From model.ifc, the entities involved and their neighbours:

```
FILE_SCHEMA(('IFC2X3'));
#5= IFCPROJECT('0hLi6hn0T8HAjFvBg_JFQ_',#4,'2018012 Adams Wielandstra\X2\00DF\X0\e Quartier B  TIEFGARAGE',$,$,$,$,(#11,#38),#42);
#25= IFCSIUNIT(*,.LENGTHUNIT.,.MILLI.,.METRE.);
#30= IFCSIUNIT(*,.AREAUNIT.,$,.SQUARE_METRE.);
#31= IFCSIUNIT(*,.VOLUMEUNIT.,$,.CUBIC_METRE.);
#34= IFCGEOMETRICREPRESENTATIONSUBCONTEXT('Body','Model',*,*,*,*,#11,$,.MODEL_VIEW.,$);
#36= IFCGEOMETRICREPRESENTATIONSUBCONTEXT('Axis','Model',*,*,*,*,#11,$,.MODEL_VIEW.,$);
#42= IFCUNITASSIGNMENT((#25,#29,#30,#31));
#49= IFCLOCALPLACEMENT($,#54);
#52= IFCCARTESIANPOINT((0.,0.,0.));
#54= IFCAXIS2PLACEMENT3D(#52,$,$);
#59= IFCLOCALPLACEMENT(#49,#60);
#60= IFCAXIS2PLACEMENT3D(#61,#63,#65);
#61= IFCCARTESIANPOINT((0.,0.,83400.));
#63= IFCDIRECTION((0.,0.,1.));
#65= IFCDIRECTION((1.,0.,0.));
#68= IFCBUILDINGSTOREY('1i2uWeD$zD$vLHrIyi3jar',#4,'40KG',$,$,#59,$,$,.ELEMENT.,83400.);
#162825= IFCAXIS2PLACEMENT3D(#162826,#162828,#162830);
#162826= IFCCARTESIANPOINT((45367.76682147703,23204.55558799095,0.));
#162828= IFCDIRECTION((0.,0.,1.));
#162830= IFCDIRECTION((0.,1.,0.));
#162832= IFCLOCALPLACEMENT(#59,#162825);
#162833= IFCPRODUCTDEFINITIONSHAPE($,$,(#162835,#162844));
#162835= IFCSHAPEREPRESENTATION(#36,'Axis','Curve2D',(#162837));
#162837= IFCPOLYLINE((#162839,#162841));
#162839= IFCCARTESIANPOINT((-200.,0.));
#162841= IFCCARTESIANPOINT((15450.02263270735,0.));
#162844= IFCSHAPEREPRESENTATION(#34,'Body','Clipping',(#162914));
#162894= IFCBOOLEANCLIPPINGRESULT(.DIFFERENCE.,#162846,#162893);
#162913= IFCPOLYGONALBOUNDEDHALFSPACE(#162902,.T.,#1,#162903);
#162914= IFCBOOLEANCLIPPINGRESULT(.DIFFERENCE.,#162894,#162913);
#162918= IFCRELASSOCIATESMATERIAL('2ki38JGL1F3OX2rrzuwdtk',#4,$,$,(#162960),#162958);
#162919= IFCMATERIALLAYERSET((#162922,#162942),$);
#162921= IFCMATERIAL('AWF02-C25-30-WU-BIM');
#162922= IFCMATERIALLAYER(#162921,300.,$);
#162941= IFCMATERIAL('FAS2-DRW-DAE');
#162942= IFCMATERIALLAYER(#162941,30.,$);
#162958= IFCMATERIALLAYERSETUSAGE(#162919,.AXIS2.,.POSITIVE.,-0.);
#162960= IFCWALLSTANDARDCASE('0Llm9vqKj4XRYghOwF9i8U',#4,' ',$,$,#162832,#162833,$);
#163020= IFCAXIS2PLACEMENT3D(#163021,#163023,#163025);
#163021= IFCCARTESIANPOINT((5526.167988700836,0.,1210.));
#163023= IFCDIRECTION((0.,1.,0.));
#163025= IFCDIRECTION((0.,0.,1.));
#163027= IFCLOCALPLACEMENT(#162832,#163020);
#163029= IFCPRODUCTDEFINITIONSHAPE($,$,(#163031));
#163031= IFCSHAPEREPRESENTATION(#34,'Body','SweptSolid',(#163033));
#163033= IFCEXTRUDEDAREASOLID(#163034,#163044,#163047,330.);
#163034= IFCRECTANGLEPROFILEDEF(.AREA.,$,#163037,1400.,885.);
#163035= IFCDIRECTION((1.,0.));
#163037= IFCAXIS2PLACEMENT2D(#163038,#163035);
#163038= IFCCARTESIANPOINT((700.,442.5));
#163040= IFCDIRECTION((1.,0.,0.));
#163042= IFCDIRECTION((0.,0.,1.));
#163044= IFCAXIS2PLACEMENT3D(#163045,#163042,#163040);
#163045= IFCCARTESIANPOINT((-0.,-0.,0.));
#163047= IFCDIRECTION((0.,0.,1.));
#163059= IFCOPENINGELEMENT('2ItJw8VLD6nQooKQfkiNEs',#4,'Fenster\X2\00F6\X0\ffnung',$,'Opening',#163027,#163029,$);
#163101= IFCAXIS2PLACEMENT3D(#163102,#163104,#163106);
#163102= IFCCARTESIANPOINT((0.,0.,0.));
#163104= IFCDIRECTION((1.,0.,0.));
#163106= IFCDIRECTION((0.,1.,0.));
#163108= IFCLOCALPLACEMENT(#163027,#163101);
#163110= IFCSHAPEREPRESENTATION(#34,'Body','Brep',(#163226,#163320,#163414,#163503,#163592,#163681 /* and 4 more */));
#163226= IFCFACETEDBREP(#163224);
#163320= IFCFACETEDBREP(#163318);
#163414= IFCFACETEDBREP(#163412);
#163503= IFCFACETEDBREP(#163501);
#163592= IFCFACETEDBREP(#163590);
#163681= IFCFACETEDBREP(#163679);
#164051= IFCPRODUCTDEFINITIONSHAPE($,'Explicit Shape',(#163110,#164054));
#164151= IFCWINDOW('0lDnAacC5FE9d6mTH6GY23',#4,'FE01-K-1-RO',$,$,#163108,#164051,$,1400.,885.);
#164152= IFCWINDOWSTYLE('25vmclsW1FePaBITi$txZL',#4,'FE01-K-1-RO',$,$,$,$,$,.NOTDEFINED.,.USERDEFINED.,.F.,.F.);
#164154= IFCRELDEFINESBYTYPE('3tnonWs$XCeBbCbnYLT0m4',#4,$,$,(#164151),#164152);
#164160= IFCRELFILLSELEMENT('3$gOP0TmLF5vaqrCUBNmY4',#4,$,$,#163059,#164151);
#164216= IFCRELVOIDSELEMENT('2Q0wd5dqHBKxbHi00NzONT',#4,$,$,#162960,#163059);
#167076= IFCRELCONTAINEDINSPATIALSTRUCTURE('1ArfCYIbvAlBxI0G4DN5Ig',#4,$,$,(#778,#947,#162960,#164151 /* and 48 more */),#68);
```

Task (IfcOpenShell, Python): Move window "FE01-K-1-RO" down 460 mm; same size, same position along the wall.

```python
import numpy as np
import ifcopenshell
import ifcopenshell.api.geometry
import ifcopenshell.util.placement
import ifcopenshell.util.unit

model = ifcopenshell.open("model.ifc")
unit_scale = ifcopenshell.util.unit.calculate_unit_scale(model)

window = model.by_id(164151)
opening = window.FillsVoids[0].RelatingOpeningElement
dz = -0.46 / unit_scale

shift = np.array([0.0, 0.0, dz])
# The window is placed relative to its opening, so it follows when the opening moves.
matrix = ifcopenshell.util.placement.get_local_placement(opening.ObjectPlacement)
matrix[:3, 3] += shift
ifcopenshell.api.geometry.edit_object_placement(
    model, product=opening, matrix=matrix, is_si=False, should_transform_children=True
)

print(f"moved by {dz * unit_scale:+.3f} m")

model.write("model_v2.ifc")
```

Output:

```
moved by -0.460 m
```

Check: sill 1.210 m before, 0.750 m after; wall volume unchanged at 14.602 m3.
